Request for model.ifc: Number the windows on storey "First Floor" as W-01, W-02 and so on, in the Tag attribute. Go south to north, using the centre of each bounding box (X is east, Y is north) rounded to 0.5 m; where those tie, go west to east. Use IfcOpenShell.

First a look at what the model holds.

```python
import ifcopenshell
import ifcopenshell.util.element
import ifcopenshell.util.placement

model = ifcopenshell.open("model.ifc")
print(model.schema)
storey = next(s for s in model.by_type("IfcBuildingStorey") if s.Name == "First Floor")
windows = [e for e in ifcopenshell.util.element.get_decomposition(storey) if e.is_a("IfcWindow")]
for e in sorted(windows, key=lambda e: e.id()):
    origin = ifcopenshell.util.placement.get_local_placement(e.ObjectPlacement)[:3, 3]
    print(e.id(), e.Tag, e.Name, origin.round(2) + 0.0, sep=" | ")
```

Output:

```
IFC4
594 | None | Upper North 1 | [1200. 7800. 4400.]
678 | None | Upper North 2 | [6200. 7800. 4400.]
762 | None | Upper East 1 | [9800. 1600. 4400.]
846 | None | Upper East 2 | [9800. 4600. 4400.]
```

```python
import ifcopenshell
import ifcopenshell.geom
import ifcopenshell.util.element
import ifcopenshell.util.shape

model = ifcopenshell.open("model.ifc")
settings = ifcopenshell.geom.settings()
settings.set("use-world-coords", True)


def centre(element):
    shape = ifcopenshell.geom.create_shape(settings, element)
    return ifcopenshell.util.shape.get_bbox_centroid(shape.geometry)


storey = next(s for s in model.by_type("IfcBuildingStorey") if s.Name == "First Floor")
windows = [e for e in ifcopenshell.util.element.get_decomposition(storey) if e.is_a("IfcWindow")]

# Insertion points can sit at a corner or the storey origin, so sort by the geometry (in metres).
centres = {e: centre(e) for e in windows}
windows.sort(key=lambda e: (round(centres[e][1] / 0.5), centres[e][0]))

for i, e in enumerate(windows, start=1):
    number = f"W-{i:02d}"
    e.Tag = number
    print(e.id(), number)

model.write("model_v2.ifc")
```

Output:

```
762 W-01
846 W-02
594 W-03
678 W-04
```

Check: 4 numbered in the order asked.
